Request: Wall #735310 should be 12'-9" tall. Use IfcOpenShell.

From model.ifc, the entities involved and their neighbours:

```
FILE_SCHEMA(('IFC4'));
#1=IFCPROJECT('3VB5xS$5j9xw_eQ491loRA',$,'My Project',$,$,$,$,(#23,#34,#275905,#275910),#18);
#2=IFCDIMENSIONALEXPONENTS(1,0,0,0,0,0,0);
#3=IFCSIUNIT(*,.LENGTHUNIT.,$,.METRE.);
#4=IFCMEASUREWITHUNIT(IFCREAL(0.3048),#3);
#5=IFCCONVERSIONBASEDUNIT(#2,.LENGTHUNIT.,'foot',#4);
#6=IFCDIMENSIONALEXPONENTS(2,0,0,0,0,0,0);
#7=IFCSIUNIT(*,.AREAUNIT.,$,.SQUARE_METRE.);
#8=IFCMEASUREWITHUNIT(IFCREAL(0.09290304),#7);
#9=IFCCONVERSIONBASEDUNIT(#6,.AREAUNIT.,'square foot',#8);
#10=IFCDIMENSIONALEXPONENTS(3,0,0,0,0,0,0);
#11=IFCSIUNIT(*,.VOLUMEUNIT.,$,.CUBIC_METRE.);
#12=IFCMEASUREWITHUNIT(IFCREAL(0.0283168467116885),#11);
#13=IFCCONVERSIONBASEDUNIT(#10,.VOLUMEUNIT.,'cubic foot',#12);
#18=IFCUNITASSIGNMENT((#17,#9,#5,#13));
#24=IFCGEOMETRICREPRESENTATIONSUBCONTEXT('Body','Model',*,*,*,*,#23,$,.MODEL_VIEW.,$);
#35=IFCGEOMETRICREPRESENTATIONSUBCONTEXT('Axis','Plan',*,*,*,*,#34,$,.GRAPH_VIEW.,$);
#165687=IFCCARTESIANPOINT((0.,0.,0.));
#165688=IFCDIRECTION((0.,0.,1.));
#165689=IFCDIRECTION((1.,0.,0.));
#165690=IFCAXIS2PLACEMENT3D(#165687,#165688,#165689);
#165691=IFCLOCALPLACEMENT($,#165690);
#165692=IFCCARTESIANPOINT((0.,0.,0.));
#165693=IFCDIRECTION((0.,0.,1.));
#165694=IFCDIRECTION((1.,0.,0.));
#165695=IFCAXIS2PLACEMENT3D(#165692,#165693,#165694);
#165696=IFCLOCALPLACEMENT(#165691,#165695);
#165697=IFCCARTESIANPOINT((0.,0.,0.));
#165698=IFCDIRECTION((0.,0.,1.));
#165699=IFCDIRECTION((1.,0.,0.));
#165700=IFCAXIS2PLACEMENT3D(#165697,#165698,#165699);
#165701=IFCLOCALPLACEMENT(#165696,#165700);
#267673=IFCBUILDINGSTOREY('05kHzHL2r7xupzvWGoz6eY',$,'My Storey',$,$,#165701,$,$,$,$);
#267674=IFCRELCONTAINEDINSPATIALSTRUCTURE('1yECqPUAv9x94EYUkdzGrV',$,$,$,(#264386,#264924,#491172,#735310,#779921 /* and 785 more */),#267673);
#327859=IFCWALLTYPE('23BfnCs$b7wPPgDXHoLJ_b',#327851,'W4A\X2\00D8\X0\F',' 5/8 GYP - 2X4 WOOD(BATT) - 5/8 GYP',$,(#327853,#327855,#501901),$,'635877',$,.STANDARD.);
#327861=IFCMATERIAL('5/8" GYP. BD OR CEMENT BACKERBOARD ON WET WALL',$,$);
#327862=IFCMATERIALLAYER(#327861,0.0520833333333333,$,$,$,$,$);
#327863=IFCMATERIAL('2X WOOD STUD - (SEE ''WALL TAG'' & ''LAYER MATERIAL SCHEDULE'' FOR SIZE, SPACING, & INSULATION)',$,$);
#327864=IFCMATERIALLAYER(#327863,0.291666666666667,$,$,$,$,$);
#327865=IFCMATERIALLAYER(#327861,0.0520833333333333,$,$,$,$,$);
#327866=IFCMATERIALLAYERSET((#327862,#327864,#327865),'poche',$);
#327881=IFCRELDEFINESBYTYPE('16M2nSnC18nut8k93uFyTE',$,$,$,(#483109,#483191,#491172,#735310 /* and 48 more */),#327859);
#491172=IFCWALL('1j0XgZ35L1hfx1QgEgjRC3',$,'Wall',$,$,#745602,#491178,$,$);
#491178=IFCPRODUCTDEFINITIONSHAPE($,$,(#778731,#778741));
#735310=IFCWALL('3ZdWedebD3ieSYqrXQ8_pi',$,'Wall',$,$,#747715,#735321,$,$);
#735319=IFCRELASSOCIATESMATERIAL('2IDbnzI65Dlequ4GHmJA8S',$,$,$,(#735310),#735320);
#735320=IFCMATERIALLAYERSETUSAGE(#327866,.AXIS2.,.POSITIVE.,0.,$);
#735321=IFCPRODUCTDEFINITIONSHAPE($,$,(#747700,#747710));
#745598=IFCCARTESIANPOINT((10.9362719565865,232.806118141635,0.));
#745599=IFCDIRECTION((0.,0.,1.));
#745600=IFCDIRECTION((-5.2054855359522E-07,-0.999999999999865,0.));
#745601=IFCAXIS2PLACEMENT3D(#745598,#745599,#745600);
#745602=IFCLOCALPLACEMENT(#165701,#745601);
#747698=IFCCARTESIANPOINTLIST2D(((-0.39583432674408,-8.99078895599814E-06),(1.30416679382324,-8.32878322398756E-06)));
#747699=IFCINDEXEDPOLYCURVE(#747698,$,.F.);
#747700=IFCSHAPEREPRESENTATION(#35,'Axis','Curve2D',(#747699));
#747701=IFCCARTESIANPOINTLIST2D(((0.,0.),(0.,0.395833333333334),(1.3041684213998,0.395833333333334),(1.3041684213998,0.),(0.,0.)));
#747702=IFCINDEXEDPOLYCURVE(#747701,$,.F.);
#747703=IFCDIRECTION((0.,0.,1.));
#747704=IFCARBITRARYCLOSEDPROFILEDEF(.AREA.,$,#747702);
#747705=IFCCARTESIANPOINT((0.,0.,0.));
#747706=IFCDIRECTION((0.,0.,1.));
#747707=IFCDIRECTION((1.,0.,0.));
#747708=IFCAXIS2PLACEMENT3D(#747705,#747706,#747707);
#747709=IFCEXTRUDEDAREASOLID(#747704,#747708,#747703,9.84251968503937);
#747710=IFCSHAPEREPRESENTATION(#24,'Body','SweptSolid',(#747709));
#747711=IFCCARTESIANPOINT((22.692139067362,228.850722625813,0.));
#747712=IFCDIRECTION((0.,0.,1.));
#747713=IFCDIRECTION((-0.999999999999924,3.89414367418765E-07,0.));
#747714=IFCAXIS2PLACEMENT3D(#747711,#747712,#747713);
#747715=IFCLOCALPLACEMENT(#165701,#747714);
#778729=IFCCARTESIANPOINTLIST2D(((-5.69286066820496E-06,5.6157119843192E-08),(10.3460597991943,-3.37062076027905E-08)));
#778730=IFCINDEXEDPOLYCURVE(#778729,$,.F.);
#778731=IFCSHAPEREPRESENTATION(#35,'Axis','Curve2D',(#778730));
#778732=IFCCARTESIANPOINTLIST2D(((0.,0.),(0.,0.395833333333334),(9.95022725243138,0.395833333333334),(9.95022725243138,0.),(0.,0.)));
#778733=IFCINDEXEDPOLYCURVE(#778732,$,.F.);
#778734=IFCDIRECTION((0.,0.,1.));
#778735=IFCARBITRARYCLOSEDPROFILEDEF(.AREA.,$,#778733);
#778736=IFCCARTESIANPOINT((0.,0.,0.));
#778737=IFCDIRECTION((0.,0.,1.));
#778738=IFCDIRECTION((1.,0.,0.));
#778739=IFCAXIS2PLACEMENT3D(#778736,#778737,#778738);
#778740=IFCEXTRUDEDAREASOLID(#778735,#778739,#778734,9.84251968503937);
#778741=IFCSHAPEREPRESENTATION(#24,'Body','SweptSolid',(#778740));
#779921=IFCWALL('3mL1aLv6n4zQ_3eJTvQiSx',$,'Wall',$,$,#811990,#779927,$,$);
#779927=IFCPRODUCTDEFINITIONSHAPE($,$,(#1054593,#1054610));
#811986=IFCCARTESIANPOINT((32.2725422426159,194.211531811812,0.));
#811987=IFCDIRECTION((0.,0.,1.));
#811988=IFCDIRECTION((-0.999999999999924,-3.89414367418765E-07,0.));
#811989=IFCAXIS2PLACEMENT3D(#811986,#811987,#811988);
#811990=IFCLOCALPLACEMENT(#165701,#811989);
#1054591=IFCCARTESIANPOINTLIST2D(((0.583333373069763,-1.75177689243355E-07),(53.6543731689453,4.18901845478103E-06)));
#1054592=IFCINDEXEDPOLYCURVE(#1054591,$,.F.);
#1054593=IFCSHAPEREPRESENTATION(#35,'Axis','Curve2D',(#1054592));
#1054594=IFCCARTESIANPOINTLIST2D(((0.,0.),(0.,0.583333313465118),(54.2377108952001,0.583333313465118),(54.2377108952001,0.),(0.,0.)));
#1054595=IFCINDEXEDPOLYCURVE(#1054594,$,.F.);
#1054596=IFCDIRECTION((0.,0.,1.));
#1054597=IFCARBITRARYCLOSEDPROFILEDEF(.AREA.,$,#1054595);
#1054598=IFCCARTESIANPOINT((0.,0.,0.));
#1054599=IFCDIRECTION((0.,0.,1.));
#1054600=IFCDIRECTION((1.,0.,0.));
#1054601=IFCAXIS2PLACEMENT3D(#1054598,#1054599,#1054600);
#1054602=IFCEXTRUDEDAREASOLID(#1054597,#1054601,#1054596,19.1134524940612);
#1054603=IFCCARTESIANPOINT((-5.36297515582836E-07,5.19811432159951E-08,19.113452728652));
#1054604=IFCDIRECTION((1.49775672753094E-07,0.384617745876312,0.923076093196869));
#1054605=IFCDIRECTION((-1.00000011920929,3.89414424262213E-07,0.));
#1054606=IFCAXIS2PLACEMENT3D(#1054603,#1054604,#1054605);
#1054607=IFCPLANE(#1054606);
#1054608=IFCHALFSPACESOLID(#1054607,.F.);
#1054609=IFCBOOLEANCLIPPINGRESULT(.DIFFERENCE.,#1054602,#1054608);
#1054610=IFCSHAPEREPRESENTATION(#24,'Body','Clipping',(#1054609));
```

```python
import ifcopenshell
import ifcopenshell.geom
import ifcopenshell.util.representation
import ifcopenshell.util.shape
import ifcopenshell.util.unit

model = ifcopenshell.open("model.ifc")
unit_scale = ifcopenshell.util.unit.calculate_unit_scale(model)
settings = ifcopenshell.geom.settings()


def volume(element):
    """Net volume in cubic metres, openings subtracted."""
    shape = ifcopenshell.geom.create_shape(settings, element)
    return ifcopenshell.util.shape.get_volume(shape.geometry)


wall = model.by_guid("3ZdWedebD3ieSYqrXQ8_pi")
before = volume(wall)

body = ifcopenshell.util.representation.get_representation(wall, "Model", "Body")
solid = body.Items[0]
old_height = solid.Depth
solid.Depth = 153 * 0.0254 / unit_scale
after = volume(wall)

print(f"height {old_height:g} -> {solid.Depth:g}, volume {before:.3f} -> {after:.3f} m3")

model.write("model_rev.ifc")
```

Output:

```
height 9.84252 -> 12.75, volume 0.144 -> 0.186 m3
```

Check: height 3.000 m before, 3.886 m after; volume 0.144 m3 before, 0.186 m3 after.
